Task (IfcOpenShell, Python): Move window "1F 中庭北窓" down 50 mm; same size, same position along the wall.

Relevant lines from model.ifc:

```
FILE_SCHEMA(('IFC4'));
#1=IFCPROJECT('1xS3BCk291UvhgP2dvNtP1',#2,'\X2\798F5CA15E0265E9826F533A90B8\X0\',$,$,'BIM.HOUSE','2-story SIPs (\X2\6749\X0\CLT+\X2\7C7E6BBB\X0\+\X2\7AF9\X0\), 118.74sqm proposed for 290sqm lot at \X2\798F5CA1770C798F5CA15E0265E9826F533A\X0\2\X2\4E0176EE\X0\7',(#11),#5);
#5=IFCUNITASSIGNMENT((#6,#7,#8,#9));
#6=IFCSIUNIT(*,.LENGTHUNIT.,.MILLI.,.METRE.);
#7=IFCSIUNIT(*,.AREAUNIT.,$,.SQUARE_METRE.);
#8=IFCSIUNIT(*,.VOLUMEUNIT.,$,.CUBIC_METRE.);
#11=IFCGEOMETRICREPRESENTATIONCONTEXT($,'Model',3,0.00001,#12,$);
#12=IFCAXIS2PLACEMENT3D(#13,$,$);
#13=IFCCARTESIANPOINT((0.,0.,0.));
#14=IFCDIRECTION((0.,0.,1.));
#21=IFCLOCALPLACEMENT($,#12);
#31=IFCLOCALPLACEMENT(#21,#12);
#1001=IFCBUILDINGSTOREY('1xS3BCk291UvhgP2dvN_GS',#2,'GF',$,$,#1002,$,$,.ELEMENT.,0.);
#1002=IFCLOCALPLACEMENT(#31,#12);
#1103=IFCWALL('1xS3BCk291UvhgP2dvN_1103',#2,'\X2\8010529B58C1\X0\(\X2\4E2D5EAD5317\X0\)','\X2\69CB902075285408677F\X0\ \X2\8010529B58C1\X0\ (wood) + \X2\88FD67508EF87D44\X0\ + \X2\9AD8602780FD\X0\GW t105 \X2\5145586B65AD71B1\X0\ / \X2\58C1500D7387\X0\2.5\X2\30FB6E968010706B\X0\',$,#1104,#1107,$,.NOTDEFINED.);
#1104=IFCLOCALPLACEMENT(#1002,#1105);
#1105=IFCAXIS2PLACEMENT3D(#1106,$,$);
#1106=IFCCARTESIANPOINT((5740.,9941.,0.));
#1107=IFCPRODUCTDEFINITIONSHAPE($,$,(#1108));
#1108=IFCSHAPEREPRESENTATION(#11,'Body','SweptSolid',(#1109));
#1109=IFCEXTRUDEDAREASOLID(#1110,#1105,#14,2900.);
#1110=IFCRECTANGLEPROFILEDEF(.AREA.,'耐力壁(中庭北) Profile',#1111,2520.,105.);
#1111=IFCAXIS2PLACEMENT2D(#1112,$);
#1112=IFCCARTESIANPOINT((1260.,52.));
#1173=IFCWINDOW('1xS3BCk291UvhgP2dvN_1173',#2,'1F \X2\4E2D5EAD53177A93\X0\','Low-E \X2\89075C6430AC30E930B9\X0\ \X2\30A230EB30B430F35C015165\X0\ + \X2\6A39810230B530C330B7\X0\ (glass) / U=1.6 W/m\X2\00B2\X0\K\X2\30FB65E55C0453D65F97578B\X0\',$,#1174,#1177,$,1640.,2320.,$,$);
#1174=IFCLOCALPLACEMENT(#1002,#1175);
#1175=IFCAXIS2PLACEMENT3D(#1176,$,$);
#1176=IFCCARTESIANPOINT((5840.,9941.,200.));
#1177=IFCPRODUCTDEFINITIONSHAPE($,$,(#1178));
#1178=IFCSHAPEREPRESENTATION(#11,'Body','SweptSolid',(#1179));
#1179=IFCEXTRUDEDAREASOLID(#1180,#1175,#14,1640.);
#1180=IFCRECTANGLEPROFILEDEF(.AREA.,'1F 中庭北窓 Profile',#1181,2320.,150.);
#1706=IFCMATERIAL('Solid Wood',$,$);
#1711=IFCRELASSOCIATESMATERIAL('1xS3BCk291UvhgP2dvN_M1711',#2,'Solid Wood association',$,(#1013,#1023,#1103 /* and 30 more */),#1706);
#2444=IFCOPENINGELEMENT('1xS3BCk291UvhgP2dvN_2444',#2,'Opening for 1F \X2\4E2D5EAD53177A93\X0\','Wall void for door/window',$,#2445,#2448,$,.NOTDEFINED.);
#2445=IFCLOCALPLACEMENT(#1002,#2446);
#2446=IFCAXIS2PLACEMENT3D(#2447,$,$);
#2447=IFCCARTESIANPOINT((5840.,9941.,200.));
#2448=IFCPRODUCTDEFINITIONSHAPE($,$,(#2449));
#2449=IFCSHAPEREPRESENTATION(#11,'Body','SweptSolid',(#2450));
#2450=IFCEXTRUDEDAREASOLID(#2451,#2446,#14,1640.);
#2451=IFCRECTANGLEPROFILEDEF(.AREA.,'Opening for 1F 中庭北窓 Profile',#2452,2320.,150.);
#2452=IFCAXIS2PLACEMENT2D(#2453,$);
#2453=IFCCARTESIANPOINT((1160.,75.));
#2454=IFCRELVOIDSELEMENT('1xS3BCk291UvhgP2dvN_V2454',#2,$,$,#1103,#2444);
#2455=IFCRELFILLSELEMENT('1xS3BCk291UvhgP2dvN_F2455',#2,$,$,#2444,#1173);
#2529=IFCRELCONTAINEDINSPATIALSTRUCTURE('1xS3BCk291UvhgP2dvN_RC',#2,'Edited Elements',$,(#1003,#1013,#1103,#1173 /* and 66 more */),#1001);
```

```python
import numpy as np
import ifcopenshell
import ifcopenshell.api.geometry
import ifcopenshell.util.placement
import ifcopenshell.util.unit

model = ifcopenshell.open("model.ifc")
unit_scale = ifcopenshell.util.unit.calculate_unit_scale(model)

window = model.by_guid("1xS3BCk291UvhgP2dvN_1173")
opening = window.FillsVoids[0].RelatingOpeningElement
dz = -50.0

shift = np.array([0.0, 0.0, dz])
# The window is not placed relative to its opening, so move both.
for product in (opening, window):
    matrix = ifcopenshell.util.placement.get_local_placement(product.ObjectPlacement)
    matrix[:3, 3] += shift
    ifcopenshell.api.geometry.edit_object_placement(model, product=product, matrix=matrix, is_si=False)

print(f"moved by {dz * unit_scale:+.3f} m")

model.write("model_v2.ifc")
```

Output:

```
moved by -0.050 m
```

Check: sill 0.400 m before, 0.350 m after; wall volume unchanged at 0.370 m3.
